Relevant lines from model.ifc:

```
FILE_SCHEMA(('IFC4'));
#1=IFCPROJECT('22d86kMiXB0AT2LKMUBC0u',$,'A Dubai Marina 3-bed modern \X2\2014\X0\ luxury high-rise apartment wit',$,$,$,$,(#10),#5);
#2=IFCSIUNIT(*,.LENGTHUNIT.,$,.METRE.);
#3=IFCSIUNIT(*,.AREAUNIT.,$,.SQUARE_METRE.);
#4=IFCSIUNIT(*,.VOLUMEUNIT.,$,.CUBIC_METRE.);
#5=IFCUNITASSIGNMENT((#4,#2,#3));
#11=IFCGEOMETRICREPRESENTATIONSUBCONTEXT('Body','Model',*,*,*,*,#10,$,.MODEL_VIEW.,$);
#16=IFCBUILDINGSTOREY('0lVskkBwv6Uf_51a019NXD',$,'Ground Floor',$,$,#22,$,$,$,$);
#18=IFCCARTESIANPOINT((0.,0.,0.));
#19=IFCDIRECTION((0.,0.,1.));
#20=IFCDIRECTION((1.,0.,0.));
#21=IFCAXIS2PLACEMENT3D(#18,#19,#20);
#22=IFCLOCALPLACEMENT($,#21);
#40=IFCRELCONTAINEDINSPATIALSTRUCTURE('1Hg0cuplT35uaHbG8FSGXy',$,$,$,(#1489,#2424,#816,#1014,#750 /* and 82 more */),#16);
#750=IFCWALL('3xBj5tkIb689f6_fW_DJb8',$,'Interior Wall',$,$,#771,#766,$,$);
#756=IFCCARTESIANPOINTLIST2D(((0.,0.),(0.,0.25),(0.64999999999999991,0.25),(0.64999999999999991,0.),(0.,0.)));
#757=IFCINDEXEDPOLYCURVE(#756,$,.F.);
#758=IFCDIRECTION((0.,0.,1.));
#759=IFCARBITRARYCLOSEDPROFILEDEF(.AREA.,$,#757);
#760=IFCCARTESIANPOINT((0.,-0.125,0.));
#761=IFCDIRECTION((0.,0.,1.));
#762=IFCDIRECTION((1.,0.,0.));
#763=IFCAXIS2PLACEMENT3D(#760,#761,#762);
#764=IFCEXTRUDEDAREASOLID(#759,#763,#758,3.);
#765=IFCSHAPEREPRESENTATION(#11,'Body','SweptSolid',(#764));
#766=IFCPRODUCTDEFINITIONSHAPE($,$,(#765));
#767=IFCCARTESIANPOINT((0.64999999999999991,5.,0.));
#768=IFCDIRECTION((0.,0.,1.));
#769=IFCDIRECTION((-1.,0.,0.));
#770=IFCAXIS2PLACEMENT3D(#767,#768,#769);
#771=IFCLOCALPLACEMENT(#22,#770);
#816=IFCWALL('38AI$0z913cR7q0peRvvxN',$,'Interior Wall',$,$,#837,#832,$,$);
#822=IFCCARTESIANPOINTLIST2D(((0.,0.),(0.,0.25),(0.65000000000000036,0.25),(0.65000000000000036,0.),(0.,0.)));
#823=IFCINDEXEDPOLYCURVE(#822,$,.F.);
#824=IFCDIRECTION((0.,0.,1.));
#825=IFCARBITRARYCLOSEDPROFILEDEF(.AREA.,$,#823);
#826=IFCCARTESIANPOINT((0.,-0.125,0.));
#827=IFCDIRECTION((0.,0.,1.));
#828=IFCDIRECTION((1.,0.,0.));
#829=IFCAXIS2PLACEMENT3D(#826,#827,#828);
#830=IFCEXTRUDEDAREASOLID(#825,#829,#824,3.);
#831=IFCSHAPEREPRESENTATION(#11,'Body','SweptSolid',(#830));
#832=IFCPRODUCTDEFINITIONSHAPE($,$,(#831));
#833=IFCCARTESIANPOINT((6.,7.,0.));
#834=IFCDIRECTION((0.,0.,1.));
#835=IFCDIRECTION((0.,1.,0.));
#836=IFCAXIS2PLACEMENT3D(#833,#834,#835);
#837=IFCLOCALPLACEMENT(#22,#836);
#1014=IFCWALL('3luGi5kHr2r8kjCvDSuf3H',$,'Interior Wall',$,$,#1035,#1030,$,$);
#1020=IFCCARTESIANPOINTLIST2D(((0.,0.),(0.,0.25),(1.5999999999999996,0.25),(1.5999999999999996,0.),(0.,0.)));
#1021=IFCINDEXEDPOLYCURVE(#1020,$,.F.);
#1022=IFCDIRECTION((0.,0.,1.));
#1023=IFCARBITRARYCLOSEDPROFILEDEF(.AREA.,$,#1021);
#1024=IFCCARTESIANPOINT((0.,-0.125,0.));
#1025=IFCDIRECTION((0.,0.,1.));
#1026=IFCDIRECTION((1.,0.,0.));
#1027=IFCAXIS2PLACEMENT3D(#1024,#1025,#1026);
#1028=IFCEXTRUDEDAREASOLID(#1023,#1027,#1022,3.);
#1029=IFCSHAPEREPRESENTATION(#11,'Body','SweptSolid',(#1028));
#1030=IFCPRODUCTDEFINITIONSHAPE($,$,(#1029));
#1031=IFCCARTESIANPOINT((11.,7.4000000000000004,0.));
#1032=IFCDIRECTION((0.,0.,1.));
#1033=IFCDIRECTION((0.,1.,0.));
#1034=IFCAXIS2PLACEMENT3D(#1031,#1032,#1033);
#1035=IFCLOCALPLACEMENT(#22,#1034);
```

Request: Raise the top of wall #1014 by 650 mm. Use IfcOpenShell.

```python
import ifcopenshell
import ifcopenshell.geom
import ifcopenshell.util.representation
import ifcopenshell.util.shape

model = ifcopenshell.open("model.ifc")
settings = ifcopenshell.geom.settings()


def volume(element):
    """Net volume in cubic metres, openings subtracted."""
    shape = ifcopenshell.geom.create_shape(settings, element)
    return ifcopenshell.util.shape.get_volume(shape.geometry)


wall = model.by_guid("3luGi5kHr2r8kjCvDSuf3H")
before = volume(wall)

body = ifcopenshell.util.representation.get_representation(wall, "Model", "Body")
solid = body.Items[0]
old_height = solid.Depth
solid.Depth += 0.65
after = volume(wall)

print(f"height {old_height:g} -> {solid.Depth:g}, volume {before:.3f} -> {after:.3f} m3")

model.write("model_v2.ifc")
```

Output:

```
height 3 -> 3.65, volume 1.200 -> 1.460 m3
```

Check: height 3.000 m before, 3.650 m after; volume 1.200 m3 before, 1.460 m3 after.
